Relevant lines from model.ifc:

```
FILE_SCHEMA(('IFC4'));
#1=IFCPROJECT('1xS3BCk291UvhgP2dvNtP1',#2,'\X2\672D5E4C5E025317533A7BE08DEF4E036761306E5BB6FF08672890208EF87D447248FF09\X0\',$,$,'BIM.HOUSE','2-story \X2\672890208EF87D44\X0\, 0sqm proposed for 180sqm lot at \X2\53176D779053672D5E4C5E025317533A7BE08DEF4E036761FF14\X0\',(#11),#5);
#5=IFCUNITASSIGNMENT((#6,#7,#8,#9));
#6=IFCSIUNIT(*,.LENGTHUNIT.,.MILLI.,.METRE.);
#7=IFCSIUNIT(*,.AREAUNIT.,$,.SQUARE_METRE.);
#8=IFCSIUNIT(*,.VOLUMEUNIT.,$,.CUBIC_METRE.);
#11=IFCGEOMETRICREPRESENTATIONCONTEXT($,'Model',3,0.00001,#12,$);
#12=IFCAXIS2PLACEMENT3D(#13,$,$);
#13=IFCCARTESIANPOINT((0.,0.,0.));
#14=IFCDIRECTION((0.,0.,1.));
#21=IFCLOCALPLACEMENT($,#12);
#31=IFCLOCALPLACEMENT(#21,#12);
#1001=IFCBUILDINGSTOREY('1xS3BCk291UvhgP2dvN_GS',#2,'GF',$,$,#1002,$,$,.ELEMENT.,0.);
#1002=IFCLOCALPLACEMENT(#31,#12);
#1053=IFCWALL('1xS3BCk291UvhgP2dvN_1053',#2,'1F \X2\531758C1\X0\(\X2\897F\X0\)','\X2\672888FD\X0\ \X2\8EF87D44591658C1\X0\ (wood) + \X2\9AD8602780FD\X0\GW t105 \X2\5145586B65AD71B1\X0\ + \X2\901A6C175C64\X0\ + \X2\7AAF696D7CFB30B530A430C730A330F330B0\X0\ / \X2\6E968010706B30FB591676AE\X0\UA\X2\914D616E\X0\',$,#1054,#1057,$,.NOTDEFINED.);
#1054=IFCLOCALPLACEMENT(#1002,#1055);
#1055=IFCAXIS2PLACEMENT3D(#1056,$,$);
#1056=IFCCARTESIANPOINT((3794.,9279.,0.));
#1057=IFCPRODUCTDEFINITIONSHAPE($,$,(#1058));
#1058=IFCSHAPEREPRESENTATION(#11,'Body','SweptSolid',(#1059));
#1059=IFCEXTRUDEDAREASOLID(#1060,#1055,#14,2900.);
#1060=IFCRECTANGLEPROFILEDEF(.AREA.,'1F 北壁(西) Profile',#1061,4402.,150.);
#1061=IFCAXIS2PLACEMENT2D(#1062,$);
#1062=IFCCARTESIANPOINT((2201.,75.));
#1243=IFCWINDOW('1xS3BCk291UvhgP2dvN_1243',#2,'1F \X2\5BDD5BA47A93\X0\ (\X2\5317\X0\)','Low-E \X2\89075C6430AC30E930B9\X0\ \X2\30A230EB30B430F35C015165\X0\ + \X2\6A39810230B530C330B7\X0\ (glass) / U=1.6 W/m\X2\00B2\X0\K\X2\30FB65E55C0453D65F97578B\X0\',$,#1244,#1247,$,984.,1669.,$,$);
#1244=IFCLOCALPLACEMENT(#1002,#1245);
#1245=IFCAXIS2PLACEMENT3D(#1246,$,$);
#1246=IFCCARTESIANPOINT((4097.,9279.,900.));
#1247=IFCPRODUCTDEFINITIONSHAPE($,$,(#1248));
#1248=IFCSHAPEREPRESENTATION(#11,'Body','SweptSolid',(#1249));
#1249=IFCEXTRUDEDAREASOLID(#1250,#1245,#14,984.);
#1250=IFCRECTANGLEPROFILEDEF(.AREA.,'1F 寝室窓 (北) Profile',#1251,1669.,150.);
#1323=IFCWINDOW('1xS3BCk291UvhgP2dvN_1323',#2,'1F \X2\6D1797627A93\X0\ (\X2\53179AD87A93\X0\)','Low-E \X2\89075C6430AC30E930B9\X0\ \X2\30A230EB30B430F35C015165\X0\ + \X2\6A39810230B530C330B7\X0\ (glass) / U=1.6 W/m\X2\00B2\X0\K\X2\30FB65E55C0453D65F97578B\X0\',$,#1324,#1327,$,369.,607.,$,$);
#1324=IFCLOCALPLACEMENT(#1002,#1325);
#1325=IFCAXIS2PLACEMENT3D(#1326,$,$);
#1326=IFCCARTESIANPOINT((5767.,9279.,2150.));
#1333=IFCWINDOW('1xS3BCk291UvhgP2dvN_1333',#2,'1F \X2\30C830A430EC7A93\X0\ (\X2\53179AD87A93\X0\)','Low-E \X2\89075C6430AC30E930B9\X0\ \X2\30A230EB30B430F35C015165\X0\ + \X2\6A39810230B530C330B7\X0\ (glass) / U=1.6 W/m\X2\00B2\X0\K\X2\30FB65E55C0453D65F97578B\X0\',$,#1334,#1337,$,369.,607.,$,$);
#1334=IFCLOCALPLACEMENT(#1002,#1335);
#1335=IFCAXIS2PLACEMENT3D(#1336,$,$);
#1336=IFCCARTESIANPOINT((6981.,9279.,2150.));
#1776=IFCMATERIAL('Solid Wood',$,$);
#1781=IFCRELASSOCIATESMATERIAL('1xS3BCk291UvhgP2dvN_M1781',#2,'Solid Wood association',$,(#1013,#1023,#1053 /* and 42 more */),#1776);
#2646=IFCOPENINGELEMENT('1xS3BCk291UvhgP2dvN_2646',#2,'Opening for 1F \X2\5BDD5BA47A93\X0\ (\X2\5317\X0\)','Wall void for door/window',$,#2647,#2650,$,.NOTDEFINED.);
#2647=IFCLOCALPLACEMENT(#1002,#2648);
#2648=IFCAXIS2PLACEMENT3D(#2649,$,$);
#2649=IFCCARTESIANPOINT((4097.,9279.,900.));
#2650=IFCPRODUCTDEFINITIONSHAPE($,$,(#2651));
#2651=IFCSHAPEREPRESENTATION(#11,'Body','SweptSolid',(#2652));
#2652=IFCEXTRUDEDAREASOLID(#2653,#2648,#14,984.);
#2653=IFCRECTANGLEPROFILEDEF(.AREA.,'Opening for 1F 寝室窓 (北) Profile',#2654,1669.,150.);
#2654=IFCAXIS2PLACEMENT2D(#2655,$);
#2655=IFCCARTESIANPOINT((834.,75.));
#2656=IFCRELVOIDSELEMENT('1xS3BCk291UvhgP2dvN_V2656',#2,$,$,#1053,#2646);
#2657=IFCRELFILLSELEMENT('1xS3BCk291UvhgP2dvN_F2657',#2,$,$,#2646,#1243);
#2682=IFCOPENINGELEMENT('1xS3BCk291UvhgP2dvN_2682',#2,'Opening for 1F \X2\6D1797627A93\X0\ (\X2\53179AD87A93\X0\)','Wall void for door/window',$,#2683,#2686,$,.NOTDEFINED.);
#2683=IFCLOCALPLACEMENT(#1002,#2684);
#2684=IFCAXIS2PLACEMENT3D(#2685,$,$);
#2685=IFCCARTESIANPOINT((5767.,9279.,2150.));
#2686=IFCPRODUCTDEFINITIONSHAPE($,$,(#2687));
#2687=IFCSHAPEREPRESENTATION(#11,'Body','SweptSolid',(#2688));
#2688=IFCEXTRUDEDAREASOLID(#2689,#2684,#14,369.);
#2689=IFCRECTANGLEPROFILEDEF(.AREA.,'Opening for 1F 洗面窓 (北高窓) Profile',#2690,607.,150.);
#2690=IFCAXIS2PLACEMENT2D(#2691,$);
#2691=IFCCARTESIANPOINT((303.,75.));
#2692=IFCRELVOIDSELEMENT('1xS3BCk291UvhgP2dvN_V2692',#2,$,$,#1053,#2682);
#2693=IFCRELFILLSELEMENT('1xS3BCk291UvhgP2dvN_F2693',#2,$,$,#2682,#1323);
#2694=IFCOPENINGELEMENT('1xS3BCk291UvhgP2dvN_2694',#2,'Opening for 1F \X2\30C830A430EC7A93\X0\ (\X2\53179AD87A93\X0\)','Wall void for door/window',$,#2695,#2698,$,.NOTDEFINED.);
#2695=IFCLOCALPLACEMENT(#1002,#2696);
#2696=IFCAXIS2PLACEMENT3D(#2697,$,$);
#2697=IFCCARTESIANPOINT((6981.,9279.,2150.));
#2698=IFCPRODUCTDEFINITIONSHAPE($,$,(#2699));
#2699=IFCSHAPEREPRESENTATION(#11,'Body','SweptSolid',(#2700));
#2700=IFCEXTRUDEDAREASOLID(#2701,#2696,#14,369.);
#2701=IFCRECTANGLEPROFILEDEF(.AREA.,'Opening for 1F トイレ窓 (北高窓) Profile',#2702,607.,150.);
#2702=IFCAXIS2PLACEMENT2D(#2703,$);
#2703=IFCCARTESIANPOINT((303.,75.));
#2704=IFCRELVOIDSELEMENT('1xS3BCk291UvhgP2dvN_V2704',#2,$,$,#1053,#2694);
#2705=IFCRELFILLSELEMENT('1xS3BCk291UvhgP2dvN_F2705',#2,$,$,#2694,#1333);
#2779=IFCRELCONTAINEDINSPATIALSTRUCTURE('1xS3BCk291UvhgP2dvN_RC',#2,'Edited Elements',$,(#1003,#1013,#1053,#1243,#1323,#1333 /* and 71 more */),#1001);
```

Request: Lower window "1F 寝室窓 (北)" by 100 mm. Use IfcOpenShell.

```python
import numpy as np
import ifcopenshell
import ifcopenshell.api.geometry
import ifcopenshell.util.placement
import ifcopenshell.util.unit

model = ifcopenshell.open("model.ifc")
unit_scale = ifcopenshell.util.unit.calculate_unit_scale(model)

window = model.by_guid("1xS3BCk291UvhgP2dvN_1243")
opening = window.FillsVoids[0].RelatingOpeningElement
dz = -0.1 / unit_scale

shift = np.array([0.0, 0.0, dz])
# The window is not placed relative to its opening, so move both.
for product in (opening, window):
    matrix = ifcopenshell.util.placement.get_local_placement(product.ObjectPlacement)
    matrix[:3, 3] += shift
    ifcopenshell.api.geometry.edit_object_placement(model, product=product, matrix=matrix, is_si=False)

print(f"moved by {dz * unit_scale:+.3f} m")

model.write("model-out.ifc")
```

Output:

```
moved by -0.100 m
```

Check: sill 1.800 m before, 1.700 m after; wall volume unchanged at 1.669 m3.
